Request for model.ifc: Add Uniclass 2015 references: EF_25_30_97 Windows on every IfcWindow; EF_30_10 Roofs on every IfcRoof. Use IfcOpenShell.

First a look at what the model holds.

```python
import ifcopenshell

model = ifcopenshell.open("model.ifc")
print(model.schema)
print("classifications:", [c.Name for c in model.by_type("IfcClassification")])
for ifc_class in ("IfcDoor", "IfcRoof", "IfcStair", "IfcWall", "IfcWindow"):
    print(ifc_class, len(model.by_type(ifc_class)))
```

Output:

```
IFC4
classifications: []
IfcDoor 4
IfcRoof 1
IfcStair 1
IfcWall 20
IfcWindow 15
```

```python
import ifcopenshell
import ifcopenshell.api.classification

model = ifcopenshell.open("model.ifc")

system = ifcopenshell.api.classification.add_classification(model, classification="Uniclass 2015")

codes = {
    "IfcWindow": ("EF_25_30_97", "Windows"),
    "IfcRoof": ("EF_30_10", "Roofs"),
}
for ifc_class, (code, name) in codes.items():
    products = model.by_type(ifc_class)
    ifcopenshell.api.classification.add_reference(
        model, products=products, classification=system, identification=code, name=name
    )
    print(code, len(products))

model.write("model_v2.ifc")
```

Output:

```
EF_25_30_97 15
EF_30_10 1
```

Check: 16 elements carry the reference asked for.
